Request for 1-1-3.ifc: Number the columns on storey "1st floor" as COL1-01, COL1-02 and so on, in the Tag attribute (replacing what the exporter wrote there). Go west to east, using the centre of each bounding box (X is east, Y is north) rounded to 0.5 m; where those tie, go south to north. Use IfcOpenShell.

First a look at what the model holds.

```python
import ifcopenshell
import ifcopenshell.util.element
import ifcopenshell.util.placement

model = ifcopenshell.open("1-1-3.ifc")
print(model.schema)
storey = next(s for s in model.by_type("IfcBuildingStorey") if s.Name == "1st floor")
columns = [e for e in ifcopenshell.util.element.get_decomposition(storey) if e.is_a("IfcColumn")]
for e in sorted(columns, key=lambda e: e.id()):
    origin = ifcopenshell.util.placement.get_local_placement(e.ObjectPlacement)[:3, 3]
    print(e.id(), e.Tag, e.Name, origin.round(2) + 0.0, sep=" | ")
```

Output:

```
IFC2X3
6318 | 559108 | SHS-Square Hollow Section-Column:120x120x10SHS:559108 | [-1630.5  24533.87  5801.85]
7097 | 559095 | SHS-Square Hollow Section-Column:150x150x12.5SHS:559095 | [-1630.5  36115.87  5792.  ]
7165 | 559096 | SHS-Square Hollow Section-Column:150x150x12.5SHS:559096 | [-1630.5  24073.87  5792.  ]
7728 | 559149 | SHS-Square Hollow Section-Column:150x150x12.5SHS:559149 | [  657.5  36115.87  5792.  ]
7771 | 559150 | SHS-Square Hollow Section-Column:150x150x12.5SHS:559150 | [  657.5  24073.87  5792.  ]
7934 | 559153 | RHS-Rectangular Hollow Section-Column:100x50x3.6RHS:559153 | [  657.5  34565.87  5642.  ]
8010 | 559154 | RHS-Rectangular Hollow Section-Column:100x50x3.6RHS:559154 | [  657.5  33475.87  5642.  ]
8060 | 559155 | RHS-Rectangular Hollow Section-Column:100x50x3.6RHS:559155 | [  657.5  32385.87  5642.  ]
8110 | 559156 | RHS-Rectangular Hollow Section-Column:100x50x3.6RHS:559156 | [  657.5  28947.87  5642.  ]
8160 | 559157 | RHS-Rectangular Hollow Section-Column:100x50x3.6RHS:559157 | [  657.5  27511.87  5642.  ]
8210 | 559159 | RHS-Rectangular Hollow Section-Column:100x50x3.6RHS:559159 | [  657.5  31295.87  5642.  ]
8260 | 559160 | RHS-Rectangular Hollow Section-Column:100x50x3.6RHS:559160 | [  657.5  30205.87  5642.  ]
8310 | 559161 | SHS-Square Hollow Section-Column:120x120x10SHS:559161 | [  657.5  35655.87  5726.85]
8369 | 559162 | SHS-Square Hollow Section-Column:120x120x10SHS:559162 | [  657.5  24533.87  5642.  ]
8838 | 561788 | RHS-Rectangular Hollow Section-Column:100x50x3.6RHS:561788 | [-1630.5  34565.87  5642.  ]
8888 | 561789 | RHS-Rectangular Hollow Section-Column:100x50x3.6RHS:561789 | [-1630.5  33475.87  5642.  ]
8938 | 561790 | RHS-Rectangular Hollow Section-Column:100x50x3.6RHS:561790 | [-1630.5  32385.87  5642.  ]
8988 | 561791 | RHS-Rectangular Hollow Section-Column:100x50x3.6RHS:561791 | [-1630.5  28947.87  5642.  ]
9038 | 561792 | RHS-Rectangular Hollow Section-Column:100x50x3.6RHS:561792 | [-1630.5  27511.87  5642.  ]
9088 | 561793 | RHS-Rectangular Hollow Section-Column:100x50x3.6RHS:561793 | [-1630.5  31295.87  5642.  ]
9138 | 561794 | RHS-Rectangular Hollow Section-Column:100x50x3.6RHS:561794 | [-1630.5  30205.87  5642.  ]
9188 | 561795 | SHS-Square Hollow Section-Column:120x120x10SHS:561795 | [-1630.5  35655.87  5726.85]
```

```python
import ifcopenshell
import ifcopenshell.geom
import ifcopenshell.util.element
import ifcopenshell.util.shape

model = ifcopenshell.open("1-1-3.ifc")
settings = ifcopenshell.geom.settings()
settings.set("use-world-coords", True)


def centre(element):
    shape = ifcopenshell.geom.create_shape(settings, element)
    return ifcopenshell.util.shape.get_bbox_centroid(shape.geometry)


storey = next(s for s in model.by_type("IfcBuildingStorey") if s.Name == "1st floor")
columns = [e for e in ifcopenshell.util.element.get_decomposition(storey) if e.is_a("IfcColumn")]

# Insertion points can sit at a corner or the storey origin, so sort by the geometry (in metres).
centres = {e: centre(e) for e in columns}
columns.sort(key=lambda e: (round(centres[e][0] / 0.5), centres[e][1]))

for i, e in enumerate(columns, start=1):
    number = f"COL1-{i:02d}"
    e.Tag = number
    print(e.id(), number)

model.write("1-1-3_edited.ifc")
```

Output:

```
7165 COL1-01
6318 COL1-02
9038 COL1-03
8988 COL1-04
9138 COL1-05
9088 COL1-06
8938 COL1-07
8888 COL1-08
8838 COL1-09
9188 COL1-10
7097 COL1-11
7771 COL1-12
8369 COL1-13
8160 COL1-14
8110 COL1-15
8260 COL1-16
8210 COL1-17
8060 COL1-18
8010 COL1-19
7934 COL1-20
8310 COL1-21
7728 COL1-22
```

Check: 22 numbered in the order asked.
